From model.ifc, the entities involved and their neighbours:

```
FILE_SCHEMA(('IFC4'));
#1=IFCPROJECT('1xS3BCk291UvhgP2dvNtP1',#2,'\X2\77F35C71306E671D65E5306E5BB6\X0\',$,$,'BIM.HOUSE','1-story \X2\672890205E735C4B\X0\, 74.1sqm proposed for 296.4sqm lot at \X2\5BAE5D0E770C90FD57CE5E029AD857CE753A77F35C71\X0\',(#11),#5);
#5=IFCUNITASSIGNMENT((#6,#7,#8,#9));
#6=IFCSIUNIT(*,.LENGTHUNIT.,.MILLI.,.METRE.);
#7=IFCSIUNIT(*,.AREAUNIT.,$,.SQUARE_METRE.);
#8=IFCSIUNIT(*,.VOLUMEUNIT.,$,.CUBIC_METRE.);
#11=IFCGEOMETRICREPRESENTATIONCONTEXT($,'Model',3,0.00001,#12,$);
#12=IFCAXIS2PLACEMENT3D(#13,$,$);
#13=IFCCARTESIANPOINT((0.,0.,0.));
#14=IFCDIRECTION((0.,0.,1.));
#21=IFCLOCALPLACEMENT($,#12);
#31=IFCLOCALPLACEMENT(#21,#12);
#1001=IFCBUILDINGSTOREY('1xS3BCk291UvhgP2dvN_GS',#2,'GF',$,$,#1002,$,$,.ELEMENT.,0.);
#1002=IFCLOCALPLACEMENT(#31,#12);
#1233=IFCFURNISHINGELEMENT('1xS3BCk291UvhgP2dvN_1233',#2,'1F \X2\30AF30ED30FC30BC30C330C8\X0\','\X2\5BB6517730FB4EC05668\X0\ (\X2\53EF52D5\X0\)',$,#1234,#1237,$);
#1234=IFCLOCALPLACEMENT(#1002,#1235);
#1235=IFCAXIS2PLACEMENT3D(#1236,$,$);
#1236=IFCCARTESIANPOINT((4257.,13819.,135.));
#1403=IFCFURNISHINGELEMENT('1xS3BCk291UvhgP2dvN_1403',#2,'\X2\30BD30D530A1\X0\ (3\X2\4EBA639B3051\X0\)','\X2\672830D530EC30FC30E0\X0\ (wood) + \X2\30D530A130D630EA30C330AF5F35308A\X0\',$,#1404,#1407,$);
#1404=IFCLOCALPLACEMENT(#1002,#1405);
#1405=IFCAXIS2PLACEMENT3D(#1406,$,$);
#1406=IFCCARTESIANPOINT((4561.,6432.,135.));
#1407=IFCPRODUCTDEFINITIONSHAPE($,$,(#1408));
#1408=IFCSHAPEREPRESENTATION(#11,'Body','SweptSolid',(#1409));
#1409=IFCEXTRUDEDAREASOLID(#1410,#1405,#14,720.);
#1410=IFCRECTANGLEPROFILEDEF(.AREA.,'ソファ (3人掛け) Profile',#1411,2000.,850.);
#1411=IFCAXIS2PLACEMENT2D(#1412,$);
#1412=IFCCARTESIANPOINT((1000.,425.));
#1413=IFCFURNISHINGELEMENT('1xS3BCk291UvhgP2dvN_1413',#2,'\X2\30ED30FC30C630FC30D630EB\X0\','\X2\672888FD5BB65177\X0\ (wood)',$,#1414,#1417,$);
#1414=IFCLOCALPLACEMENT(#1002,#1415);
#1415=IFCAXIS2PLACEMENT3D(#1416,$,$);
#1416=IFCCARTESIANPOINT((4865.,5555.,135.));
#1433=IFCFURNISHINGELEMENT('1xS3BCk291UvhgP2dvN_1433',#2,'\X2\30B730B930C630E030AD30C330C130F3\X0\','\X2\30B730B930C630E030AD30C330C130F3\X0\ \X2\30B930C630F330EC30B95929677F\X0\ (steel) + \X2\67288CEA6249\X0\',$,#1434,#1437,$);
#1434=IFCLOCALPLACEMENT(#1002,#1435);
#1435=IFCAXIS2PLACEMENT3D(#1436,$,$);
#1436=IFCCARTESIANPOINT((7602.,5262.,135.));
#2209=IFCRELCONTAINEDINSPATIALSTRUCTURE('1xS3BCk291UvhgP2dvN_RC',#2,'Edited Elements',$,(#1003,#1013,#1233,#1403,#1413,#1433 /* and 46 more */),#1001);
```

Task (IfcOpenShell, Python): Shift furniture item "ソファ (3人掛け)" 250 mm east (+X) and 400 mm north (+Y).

```python
import ifcopenshell
import ifcopenshell.api.geometry
import ifcopenshell.util.placement

model = ifcopenshell.open("model.ifc")

item = model.by_id(1403)
matrix = ifcopenshell.util.placement.get_local_placement(item.ObjectPlacement)
matrix[0, 3] += 250.0
matrix[1, 3] += 400.0
ifcopenshell.api.geometry.edit_object_placement(model, product=item, matrix=matrix, is_si=False)

print(ifcopenshell.util.placement.get_local_placement(item.ObjectPlacement).round(3) + 0.0)

model.write("model_v2.ifc")
```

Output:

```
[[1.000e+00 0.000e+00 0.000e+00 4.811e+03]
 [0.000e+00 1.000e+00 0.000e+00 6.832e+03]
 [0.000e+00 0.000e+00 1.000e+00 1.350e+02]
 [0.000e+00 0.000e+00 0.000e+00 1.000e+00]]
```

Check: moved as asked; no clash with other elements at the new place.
